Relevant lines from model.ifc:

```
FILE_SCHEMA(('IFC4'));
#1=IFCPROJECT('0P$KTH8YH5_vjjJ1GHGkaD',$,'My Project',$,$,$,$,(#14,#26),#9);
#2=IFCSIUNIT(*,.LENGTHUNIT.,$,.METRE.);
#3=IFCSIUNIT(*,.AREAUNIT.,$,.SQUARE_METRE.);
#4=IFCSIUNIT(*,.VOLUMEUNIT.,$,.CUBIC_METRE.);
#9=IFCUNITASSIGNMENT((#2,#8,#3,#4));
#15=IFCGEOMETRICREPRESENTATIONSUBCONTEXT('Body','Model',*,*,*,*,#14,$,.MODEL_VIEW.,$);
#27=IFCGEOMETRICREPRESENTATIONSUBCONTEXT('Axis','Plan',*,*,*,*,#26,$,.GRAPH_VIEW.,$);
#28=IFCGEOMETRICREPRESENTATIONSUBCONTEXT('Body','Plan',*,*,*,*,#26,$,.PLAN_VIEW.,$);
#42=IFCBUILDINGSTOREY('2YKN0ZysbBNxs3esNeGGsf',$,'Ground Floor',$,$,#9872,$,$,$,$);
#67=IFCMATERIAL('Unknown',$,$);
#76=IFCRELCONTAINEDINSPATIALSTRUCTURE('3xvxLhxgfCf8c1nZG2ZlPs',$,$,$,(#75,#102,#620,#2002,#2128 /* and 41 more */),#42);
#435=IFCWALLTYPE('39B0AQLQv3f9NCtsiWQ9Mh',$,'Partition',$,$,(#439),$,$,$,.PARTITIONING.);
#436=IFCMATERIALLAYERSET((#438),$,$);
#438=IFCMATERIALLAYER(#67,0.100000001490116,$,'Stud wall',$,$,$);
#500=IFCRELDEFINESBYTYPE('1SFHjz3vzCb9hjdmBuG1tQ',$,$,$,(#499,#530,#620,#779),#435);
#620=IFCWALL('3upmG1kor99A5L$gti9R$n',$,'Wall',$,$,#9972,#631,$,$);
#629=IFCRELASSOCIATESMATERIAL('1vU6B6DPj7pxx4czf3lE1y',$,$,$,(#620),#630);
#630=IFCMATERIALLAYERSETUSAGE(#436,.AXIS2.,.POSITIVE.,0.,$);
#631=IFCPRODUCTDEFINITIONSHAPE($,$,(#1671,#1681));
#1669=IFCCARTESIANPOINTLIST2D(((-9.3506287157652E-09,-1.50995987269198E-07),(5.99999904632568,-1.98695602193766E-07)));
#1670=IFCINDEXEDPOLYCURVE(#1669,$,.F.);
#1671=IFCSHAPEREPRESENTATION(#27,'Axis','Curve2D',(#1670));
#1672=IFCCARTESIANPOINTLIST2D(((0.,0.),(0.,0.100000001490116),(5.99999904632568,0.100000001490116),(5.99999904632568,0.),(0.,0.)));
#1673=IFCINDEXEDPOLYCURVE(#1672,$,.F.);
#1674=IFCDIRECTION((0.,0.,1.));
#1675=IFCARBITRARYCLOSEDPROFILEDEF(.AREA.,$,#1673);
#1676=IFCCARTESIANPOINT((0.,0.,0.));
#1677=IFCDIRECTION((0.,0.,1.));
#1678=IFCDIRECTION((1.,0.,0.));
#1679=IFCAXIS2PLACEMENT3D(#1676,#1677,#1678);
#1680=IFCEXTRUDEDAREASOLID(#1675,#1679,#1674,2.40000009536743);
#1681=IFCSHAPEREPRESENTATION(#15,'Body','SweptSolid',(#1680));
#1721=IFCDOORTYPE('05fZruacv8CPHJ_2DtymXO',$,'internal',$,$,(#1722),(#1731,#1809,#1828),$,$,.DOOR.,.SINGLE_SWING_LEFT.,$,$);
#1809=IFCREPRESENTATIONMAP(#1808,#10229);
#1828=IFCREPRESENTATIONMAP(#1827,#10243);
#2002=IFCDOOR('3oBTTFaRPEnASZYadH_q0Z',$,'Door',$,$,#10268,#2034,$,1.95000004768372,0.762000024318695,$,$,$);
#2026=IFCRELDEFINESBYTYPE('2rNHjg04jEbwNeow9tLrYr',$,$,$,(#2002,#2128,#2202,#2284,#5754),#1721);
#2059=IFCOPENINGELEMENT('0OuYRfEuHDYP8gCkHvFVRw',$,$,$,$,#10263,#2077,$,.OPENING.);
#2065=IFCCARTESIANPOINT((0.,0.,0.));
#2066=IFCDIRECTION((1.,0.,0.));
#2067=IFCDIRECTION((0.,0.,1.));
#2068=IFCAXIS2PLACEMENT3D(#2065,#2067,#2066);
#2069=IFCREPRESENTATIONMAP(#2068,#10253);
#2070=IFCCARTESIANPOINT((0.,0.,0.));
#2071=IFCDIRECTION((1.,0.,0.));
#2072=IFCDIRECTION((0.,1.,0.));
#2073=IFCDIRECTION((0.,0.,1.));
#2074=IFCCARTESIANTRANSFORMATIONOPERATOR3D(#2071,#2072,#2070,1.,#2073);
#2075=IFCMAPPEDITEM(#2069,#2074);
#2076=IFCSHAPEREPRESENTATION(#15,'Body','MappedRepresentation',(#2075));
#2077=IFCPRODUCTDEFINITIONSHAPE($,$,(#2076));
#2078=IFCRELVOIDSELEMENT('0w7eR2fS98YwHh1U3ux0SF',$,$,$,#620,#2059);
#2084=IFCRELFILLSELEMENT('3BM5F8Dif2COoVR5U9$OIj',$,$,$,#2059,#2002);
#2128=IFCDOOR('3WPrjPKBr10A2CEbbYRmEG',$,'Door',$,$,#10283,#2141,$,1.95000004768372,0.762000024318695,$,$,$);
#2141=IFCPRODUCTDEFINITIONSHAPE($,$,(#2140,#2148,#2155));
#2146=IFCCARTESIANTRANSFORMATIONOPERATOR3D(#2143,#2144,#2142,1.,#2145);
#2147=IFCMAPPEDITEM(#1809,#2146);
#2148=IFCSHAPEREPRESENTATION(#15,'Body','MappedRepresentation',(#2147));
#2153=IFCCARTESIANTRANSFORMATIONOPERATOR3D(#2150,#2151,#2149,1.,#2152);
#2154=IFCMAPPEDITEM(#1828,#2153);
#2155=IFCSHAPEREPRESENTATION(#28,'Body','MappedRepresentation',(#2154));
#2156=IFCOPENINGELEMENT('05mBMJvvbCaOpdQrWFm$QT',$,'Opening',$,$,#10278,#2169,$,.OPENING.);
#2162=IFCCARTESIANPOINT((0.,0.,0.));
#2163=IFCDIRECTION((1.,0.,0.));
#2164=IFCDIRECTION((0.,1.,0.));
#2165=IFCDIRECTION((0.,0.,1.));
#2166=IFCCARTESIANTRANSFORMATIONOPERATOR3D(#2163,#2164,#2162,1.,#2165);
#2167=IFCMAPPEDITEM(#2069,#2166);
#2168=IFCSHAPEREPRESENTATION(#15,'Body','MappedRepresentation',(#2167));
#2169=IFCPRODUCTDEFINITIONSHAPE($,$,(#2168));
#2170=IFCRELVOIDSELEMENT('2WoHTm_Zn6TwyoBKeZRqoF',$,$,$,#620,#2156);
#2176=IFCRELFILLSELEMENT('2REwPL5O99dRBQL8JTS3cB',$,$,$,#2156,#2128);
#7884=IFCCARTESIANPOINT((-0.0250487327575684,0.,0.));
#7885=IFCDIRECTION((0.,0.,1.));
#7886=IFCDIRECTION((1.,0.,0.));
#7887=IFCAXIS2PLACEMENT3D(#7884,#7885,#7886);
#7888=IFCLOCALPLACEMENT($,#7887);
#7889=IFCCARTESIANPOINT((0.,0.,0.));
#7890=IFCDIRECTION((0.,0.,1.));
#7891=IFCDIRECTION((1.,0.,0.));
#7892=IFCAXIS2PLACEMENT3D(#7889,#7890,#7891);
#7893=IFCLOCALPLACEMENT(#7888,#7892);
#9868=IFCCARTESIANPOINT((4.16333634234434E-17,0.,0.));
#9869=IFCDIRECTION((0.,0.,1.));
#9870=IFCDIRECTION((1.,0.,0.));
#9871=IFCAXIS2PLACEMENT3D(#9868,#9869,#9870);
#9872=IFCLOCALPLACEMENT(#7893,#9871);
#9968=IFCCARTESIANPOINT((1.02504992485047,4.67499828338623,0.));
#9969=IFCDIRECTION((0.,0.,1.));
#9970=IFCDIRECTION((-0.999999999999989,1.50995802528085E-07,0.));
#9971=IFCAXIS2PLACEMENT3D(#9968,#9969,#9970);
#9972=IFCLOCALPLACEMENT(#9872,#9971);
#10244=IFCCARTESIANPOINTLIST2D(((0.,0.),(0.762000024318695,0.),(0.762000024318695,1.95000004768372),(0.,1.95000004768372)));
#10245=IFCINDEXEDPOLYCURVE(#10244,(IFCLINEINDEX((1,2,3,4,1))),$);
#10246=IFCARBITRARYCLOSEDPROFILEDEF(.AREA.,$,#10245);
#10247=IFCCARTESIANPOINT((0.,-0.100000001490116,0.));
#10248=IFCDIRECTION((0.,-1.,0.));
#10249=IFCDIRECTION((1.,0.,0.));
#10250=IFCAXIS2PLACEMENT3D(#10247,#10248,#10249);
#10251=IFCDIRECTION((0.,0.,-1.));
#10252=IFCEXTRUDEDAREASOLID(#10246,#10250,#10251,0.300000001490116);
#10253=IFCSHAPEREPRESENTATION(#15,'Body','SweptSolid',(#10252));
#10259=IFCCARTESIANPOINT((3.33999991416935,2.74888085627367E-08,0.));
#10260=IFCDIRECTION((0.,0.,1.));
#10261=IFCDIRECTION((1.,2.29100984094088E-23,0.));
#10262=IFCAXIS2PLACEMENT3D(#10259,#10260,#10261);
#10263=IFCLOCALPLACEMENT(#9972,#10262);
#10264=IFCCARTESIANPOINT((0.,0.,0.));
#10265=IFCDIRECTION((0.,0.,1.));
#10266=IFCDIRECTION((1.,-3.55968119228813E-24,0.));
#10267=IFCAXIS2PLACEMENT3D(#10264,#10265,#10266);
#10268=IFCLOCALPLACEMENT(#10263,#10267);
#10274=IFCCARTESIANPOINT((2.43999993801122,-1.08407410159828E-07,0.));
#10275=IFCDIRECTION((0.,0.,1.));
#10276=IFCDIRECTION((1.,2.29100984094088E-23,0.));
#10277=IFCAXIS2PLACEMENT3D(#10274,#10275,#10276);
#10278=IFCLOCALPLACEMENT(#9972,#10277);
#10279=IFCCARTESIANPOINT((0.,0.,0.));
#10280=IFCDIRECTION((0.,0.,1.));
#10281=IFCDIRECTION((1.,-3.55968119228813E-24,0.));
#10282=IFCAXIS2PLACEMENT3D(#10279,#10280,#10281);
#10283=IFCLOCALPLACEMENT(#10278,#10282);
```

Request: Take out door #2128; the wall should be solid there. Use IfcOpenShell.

```python
import ifcopenshell
import ifcopenshell.api.feature
import ifcopenshell.api.root
import ifcopenshell.geom
import ifcopenshell.util.shape

model = ifcopenshell.open("model.ifc")
settings = ifcopenshell.geom.settings()


def volume(element):
    """Net volume in cubic metres, openings subtracted."""
    shape = ifcopenshell.geom.create_shape(settings, element)
    return ifcopenshell.util.shape.get_volume(shape.geometry)


door = model.by_guid("3WPrjPKBr10A2CEbbYRmEG")
opening = door.FillsVoids[0].RelatingOpeningElement
wall = opening.VoidsElements[0].RelatingBuildingElement
before = volume(wall)

ifcopenshell.api.root.remove_product(model, product=door)
ifcopenshell.api.feature.remove_feature(model, feature=opening)

after = volume(wall)

print(f"wall volume {before:.3f} -> {after:.3f} m3")

model.write("model_edited.ifc")
```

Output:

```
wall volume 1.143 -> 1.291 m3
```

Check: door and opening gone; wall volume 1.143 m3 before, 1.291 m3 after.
